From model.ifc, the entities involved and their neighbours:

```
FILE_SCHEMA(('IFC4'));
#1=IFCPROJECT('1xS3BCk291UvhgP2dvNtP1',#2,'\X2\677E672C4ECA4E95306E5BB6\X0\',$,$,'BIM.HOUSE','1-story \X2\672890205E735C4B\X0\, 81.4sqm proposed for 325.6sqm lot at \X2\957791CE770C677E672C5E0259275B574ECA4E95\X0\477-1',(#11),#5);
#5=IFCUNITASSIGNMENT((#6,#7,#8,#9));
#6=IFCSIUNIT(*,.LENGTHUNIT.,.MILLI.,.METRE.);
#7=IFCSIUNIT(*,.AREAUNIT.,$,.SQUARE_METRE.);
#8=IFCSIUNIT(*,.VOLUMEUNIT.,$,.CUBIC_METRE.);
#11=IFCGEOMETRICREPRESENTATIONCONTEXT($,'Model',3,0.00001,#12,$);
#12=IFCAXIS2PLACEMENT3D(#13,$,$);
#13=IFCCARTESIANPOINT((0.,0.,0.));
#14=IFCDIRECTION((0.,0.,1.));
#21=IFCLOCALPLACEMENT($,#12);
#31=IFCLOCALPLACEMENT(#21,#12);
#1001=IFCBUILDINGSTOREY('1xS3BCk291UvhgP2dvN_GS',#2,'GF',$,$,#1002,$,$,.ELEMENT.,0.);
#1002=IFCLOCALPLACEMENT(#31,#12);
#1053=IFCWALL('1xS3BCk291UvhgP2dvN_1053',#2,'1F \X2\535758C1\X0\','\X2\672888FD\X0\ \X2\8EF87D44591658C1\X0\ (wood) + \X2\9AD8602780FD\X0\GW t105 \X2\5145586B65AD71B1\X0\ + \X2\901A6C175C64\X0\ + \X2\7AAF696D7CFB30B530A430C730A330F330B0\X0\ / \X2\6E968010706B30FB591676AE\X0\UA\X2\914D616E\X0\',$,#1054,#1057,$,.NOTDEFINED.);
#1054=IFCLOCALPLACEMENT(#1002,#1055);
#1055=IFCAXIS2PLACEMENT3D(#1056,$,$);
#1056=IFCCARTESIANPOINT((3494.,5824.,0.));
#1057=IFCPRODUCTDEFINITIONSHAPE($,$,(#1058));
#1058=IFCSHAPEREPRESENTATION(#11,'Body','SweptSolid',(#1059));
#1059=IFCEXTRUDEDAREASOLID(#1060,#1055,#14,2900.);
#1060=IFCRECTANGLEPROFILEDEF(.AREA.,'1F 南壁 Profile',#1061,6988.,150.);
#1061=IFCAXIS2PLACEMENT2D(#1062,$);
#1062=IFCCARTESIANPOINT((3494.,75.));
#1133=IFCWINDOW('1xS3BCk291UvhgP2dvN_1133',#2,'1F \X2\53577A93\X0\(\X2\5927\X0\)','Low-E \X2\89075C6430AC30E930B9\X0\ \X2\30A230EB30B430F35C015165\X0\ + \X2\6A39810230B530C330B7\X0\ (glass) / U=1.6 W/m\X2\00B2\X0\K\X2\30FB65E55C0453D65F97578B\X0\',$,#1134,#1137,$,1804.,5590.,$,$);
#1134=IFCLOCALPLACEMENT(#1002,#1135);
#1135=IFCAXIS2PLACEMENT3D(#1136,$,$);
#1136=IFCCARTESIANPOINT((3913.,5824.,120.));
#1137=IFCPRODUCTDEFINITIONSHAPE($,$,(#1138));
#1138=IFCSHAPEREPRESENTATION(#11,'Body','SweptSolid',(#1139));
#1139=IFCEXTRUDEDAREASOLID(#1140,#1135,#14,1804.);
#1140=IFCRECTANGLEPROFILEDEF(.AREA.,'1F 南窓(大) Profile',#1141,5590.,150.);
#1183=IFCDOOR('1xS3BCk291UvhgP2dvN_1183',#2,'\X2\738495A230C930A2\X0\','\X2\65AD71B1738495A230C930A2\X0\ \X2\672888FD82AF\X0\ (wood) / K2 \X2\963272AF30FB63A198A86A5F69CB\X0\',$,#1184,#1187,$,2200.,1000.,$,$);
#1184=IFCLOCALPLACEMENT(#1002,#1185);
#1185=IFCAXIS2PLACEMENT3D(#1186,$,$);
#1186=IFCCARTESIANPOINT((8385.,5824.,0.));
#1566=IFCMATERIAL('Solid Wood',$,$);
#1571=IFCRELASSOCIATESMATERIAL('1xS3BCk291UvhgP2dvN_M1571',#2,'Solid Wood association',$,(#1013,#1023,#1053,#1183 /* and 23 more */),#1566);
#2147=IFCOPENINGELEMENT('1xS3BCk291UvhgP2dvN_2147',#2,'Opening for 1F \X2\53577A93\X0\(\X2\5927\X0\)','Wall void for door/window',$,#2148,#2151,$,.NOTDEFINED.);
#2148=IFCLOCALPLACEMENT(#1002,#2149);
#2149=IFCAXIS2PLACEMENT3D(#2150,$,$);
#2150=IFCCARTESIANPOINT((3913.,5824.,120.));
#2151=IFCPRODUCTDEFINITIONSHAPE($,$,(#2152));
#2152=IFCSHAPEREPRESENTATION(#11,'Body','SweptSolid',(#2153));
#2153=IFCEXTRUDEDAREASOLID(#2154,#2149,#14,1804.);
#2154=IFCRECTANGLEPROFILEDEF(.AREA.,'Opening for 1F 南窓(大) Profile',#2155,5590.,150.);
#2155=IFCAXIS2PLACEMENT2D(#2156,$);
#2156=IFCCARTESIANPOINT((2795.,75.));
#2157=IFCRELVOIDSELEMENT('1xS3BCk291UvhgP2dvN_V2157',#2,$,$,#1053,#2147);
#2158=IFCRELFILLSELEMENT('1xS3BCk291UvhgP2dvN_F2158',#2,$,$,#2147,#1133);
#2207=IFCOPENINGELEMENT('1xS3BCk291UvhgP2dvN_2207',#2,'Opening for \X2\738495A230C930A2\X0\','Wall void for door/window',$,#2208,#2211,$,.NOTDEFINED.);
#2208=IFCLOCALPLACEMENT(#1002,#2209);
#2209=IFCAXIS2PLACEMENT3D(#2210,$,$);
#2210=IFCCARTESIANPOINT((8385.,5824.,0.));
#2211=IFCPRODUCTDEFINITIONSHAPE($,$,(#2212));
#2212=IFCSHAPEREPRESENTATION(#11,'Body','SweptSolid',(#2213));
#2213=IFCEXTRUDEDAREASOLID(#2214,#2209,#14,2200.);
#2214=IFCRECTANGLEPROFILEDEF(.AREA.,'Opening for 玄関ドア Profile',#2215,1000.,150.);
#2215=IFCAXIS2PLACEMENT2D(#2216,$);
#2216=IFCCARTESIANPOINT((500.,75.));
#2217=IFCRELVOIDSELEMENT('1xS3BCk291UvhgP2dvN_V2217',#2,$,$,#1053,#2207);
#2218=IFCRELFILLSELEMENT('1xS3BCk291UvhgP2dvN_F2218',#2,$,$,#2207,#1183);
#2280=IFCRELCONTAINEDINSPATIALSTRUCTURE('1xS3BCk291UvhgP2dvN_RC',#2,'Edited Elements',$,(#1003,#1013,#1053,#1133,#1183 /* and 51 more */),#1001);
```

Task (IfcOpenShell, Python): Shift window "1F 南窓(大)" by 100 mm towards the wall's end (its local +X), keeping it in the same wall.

```python
import ifcopenshell
import ifcopenshell.api.geometry
import ifcopenshell.util.placement
import ifcopenshell.util.unit

model = ifcopenshell.open("model.ifc")
unit_scale = ifcopenshell.util.unit.calculate_unit_scale(model)

window = model.by_guid("1xS3BCk291UvhgP2dvN_1133")
opening = window.FillsVoids[0].RelatingOpeningElement
wall = opening.VoidsElements[0].RelatingBuildingElement

wall_matrix = ifcopenshell.util.placement.get_local_placement(wall.ObjectPlacement)
shift = wall_matrix[:3, 0] * 0.1 / unit_scale
before = ifcopenshell.util.placement.get_local_placement(window.ObjectPlacement)[:3, 3].copy()

# The window is not placed relative to its opening, so move both.
for product in (opening, window):
    matrix = ifcopenshell.util.placement.get_local_placement(product.ObjectPlacement)
    matrix[:3, 3] += shift
    ifcopenshell.api.geometry.edit_object_placement(model, product=product, matrix=matrix, is_si=False)

after = ifcopenshell.util.placement.get_local_placement(window.ObjectPlacement)[:3, 3]
print("window moved by", (after - before).round(3) + 0.0)

model.write("model_v2.ifc")
```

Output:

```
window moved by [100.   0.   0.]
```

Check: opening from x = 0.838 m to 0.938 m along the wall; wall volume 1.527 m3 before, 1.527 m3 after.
